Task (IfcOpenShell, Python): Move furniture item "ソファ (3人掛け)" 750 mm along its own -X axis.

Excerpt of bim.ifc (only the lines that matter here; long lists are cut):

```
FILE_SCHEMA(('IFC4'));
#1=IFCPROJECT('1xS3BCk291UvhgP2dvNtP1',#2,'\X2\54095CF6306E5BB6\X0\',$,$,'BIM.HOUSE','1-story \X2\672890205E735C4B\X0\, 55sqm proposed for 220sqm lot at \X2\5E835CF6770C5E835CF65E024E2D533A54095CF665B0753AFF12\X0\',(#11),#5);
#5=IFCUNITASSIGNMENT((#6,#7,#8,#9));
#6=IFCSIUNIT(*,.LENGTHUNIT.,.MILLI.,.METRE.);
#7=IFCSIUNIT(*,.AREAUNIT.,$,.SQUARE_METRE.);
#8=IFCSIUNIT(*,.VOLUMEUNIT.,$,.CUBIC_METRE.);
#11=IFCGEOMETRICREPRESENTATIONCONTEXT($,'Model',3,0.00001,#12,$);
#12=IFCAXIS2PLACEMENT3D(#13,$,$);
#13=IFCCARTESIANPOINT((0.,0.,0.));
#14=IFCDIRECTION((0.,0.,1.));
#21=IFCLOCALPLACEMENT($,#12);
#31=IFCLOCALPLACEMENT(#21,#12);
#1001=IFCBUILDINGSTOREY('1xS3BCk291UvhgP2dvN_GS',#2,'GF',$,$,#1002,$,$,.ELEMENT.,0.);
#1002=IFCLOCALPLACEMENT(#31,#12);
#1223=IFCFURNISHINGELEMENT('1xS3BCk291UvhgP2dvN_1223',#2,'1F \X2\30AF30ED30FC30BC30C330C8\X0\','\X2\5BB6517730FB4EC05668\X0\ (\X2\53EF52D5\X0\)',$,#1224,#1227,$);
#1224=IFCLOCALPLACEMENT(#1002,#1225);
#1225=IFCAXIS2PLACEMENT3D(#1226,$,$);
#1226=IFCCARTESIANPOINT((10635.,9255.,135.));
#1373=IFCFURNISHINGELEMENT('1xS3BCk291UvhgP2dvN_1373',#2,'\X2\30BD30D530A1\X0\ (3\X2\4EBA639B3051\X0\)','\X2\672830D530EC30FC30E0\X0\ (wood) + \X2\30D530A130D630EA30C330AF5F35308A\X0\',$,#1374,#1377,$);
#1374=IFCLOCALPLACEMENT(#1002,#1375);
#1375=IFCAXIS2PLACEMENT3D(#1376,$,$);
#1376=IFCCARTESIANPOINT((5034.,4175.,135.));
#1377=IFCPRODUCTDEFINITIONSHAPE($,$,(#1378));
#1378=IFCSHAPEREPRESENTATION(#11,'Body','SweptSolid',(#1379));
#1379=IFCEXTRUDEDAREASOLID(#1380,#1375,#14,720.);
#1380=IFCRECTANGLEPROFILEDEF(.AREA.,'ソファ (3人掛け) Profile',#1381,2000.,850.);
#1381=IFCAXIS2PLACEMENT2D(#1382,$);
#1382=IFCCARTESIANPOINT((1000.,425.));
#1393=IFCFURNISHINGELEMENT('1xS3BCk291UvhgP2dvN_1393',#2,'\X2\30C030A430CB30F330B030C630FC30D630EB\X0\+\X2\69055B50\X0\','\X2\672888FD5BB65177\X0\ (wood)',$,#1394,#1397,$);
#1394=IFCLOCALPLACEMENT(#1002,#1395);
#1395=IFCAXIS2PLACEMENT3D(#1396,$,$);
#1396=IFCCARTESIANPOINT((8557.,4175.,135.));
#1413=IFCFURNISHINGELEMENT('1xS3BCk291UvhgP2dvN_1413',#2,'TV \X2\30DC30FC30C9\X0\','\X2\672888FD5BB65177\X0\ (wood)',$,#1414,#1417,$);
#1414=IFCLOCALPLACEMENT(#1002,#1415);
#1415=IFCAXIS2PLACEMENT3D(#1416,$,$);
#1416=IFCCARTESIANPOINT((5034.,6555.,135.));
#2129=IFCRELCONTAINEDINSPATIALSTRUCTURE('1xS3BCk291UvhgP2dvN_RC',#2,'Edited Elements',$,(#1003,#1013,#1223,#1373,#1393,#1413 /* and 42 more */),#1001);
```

```python
import ifcopenshell
import ifcopenshell.api.geometry
import ifcopenshell.util.placement
import ifcopenshell.util.unit

model = ifcopenshell.open("bim.ifc")
unit_scale = ifcopenshell.util.unit.calculate_unit_scale(model)

item = model.by_guid("1xS3BCk291UvhgP2dvN_1373")
matrix = ifcopenshell.util.placement.get_local_placement(item.ObjectPlacement)
matrix[:3, 3] -= matrix[:3, 0] * 0.75 / unit_scale
ifcopenshell.api.geometry.edit_object_placement(model, product=item, matrix=matrix, is_si=False)

print(ifcopenshell.util.placement.get_local_placement(item.ObjectPlacement).round(3) + 0.0)

model.write("bim_updated.ifc")
```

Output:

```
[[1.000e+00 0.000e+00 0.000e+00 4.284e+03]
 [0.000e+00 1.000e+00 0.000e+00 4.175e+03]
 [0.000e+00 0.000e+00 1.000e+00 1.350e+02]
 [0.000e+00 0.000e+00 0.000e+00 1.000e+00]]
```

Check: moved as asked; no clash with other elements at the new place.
